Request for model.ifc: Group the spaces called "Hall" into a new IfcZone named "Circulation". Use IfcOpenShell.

First a look at what the model holds.

```python
import ifcopenshell

model = ifcopenshell.open("model.ifc")
print(model.schema)
seen = {}
for space in model.by_type("IfcSpace"):
    seen[space.LongName] = seen.get(space.LongName, 0) + 1
for name, count in sorted(seen.items(), key=str):
    print(count, "x", name)
print("zones:", [z.Name for z in model.by_type("IfcZone")][:20])
```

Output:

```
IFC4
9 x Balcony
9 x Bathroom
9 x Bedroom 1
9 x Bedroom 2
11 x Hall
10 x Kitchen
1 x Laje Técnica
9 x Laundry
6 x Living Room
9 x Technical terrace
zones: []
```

```python
import ifcopenshell
import ifcopenshell.api.group
import ifcopenshell.api.root

model = ifcopenshell.open("model.ifc")

names = {"Hall"}
spaces = [s for s in model.by_type("IfcSpace") if s.LongName in names]

zone = ifcopenshell.api.root.create_entity(model, ifc_class="IfcZone", name="Circulation")
ifcopenshell.api.group.assign_group(model, products=spaces, group=zone)
print(len(spaces), "spaces in", zone.Name)

model.write("model_rev.ifc")
```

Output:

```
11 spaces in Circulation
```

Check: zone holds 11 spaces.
